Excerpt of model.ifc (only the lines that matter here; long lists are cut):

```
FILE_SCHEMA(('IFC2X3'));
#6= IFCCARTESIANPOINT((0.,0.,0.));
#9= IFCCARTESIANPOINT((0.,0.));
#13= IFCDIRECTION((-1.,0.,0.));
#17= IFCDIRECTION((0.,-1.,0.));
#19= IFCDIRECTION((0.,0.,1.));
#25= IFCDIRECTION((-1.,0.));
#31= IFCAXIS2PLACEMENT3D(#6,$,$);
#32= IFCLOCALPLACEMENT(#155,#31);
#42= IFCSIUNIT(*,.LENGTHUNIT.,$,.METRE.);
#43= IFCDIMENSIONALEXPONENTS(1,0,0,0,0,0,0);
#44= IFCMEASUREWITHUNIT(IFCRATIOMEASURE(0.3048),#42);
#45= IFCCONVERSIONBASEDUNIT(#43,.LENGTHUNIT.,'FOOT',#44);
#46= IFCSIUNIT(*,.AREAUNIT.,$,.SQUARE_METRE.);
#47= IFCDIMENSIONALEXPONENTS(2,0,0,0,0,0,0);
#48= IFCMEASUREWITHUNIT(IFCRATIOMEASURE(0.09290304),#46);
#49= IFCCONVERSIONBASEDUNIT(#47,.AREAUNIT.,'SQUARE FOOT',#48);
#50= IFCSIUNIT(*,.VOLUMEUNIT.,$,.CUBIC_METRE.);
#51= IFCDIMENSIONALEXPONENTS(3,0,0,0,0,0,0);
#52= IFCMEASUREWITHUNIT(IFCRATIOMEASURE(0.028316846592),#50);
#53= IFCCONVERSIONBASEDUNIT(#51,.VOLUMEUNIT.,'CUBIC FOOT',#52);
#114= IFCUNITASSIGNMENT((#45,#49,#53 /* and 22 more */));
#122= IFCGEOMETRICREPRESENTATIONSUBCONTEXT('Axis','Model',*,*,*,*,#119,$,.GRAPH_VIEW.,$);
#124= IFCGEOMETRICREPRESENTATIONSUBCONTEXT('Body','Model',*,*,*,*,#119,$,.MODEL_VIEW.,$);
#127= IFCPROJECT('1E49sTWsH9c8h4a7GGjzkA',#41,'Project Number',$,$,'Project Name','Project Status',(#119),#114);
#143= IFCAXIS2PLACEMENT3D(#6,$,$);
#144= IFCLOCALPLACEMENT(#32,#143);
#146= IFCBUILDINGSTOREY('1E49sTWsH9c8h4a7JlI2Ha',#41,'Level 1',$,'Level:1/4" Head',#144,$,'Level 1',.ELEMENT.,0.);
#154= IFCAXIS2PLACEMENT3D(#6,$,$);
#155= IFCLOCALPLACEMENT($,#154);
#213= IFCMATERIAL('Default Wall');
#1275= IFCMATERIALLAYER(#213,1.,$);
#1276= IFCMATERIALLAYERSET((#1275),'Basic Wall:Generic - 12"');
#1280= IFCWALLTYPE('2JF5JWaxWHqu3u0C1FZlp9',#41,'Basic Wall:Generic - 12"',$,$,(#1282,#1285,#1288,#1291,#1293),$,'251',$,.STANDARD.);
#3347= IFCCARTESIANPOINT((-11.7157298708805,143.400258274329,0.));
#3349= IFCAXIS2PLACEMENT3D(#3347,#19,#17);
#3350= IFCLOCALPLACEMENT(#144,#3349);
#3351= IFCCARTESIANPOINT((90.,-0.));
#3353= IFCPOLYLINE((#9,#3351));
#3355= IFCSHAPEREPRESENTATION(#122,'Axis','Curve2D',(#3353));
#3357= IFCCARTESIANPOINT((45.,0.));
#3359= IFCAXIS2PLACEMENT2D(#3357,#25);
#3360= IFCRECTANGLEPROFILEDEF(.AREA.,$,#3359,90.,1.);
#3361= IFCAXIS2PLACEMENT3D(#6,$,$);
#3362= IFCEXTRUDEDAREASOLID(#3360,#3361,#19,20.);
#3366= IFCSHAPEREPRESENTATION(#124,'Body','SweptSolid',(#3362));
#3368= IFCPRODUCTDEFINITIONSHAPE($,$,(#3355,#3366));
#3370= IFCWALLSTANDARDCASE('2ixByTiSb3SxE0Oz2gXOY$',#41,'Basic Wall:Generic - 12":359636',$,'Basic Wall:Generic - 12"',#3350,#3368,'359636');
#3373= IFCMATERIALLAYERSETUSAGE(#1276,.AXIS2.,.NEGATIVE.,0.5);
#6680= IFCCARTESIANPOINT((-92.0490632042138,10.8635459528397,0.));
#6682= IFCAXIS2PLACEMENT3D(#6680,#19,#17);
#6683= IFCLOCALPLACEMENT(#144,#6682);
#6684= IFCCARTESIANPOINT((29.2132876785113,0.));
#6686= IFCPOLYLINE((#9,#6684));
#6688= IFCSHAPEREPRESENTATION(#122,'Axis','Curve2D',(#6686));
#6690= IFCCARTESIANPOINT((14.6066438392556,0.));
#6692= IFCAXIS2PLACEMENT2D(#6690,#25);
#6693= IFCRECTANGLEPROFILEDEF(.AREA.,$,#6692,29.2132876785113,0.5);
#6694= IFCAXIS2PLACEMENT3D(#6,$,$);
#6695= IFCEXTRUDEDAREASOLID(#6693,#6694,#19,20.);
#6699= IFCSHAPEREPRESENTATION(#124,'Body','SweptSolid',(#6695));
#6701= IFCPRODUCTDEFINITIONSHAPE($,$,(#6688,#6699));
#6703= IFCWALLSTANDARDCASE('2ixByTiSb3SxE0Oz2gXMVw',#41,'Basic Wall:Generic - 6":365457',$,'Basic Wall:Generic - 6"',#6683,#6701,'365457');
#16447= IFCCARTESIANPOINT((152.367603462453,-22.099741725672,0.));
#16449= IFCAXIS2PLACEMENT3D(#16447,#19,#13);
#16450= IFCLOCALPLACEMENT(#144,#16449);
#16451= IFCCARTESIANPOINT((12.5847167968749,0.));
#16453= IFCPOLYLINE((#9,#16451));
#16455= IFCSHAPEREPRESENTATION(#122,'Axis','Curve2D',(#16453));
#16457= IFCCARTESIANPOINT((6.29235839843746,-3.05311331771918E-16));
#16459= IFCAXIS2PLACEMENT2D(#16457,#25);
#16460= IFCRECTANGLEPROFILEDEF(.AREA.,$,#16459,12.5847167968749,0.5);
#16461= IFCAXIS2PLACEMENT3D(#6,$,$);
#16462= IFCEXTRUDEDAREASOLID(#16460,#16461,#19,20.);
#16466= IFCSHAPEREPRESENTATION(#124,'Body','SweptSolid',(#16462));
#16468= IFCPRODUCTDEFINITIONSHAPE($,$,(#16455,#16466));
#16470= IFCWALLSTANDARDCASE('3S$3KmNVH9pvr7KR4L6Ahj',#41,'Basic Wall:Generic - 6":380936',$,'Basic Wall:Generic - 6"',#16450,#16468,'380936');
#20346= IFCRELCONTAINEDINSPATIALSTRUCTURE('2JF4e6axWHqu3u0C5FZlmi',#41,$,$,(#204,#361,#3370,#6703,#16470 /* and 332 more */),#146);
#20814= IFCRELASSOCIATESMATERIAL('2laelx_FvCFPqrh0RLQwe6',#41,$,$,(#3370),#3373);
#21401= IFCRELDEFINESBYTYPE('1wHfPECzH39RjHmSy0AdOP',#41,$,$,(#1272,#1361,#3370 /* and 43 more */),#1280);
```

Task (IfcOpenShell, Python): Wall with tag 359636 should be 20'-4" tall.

```python
import ifcopenshell
import ifcopenshell.geom
import ifcopenshell.util.representation
import ifcopenshell.util.shape
import ifcopenshell.util.unit

model = ifcopenshell.open("model.ifc")
unit_scale = ifcopenshell.util.unit.calculate_unit_scale(model)
settings = ifcopenshell.geom.settings()


def volume(element):
    """Net volume in cubic metres, openings subtracted."""
    shape = ifcopenshell.geom.create_shape(settings, element)
    return ifcopenshell.util.shape.get_volume(shape.geometry)


wall = model.by_guid("2ixByTiSb3SxE0Oz2gXOY$")
before = volume(wall)

body = ifcopenshell.util.representation.get_representation(wall, "Model", "Body")
solid = body.Items[0]
old_height = solid.Depth
solid.Depth = 244 * 0.0254 / unit_scale
after = volume(wall)

print(f"height {old_height:g} -> {solid.Depth:g}, volume {before:.3f} -> {after:.3f} m3")

model.write("model_updated.ifc")
```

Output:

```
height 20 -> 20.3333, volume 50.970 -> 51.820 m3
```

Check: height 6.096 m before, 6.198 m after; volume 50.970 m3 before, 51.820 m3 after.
